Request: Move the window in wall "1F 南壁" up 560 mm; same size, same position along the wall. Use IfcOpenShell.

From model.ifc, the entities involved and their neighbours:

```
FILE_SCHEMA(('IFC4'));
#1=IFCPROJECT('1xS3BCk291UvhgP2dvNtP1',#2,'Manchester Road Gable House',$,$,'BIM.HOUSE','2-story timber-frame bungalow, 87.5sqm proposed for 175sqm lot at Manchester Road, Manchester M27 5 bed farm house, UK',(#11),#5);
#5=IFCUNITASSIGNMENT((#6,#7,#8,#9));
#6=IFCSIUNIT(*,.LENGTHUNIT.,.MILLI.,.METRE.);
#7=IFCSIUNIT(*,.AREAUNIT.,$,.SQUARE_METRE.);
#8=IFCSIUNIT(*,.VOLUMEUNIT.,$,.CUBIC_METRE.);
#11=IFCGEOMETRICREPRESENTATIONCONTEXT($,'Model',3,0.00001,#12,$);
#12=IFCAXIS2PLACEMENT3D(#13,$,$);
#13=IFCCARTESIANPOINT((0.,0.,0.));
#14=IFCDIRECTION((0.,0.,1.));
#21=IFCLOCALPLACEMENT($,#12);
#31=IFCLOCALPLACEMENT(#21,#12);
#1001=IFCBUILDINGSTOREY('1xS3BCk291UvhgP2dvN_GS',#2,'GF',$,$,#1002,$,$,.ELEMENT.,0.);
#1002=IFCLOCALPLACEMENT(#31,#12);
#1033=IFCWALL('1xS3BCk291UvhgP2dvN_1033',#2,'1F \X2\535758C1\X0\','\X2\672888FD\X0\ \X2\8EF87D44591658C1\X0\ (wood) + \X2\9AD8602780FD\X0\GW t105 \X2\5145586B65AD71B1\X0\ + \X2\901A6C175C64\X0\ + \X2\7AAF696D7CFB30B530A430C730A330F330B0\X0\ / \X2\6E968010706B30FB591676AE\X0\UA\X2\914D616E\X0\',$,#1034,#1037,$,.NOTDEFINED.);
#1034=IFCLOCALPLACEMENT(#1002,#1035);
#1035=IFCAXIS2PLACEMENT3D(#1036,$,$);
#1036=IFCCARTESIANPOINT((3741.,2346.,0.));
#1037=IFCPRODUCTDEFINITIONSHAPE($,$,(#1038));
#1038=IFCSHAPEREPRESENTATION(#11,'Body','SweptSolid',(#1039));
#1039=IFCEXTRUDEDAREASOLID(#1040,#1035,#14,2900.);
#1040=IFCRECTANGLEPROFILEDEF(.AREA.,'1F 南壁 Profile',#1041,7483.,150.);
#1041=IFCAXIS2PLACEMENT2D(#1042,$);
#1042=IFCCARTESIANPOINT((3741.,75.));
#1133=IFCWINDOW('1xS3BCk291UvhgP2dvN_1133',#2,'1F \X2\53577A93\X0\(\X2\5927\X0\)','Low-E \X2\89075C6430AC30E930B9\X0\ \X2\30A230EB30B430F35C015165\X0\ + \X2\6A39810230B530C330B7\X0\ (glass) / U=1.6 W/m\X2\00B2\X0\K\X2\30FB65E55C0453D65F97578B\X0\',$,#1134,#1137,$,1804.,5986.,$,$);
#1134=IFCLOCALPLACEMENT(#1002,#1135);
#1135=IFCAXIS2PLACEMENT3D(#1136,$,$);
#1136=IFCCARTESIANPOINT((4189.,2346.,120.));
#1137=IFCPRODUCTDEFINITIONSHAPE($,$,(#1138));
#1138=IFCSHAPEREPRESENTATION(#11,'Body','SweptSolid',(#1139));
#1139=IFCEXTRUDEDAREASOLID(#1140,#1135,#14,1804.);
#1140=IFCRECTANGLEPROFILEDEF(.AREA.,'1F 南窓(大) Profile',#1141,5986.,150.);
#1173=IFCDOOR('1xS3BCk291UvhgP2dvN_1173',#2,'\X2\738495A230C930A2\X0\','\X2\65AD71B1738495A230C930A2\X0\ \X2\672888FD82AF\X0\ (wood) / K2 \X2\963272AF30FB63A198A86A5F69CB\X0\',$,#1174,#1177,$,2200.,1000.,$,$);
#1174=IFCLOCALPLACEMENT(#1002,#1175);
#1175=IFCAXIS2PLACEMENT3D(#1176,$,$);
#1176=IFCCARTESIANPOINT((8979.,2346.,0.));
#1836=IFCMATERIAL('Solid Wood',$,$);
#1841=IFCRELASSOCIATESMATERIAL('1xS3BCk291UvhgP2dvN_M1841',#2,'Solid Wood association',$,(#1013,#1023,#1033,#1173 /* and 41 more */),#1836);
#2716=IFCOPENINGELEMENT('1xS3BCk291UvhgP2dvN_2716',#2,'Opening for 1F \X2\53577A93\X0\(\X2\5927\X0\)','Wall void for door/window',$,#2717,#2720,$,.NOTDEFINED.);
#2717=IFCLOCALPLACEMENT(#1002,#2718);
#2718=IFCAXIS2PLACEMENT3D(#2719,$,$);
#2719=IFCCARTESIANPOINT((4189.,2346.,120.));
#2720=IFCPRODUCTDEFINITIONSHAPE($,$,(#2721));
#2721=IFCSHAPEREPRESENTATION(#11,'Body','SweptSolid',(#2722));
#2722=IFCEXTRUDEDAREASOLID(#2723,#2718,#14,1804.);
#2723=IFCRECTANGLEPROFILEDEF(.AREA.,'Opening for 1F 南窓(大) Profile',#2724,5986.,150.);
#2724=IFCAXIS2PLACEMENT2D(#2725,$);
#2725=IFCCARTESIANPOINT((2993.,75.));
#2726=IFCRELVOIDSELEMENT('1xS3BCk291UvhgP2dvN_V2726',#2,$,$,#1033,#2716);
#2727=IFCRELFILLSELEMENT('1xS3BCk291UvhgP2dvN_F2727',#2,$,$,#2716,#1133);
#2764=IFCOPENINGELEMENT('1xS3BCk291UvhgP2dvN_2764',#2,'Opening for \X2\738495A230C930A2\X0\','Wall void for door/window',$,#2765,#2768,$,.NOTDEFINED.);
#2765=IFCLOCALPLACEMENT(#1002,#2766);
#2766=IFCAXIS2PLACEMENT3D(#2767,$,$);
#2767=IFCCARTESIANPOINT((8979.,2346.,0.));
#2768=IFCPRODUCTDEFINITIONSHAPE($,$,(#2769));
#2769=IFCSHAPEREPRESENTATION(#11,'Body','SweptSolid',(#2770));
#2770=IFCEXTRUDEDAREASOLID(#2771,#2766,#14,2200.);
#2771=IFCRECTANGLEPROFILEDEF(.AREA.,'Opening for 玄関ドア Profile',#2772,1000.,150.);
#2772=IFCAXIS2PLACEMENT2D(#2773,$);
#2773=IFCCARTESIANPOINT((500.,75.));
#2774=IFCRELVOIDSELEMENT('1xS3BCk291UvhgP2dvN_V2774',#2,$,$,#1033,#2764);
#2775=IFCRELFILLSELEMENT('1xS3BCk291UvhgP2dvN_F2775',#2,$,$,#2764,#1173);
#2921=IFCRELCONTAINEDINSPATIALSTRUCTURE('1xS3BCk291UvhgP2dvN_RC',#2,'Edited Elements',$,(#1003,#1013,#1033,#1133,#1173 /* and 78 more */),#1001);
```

```python
import numpy as np
import ifcopenshell
import ifcopenshell.api.geometry
import ifcopenshell.util.placement
import ifcopenshell.util.unit

model = ifcopenshell.open("model.ifc")
unit_scale = ifcopenshell.util.unit.calculate_unit_scale(model)

window = model.by_guid("1xS3BCk291UvhgP2dvN_1133")
opening = window.FillsVoids[0].RelatingOpeningElement
dz = 560.0

shift = np.array([0.0, 0.0, dz])
# The window is not placed relative to its opening, so move both.
for product in (opening, window):
    matrix = ifcopenshell.util.placement.get_local_placement(product.ObjectPlacement)
    matrix[:3, 3] += shift
    ifcopenshell.api.geometry.edit_object_placement(model, product=product, matrix=matrix, is_si=False)

print(f"moved by {dz * unit_scale:+.3f} m")

model.write("model_v2.ifc")
```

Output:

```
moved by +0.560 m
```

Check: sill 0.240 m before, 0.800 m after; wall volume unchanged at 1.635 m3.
